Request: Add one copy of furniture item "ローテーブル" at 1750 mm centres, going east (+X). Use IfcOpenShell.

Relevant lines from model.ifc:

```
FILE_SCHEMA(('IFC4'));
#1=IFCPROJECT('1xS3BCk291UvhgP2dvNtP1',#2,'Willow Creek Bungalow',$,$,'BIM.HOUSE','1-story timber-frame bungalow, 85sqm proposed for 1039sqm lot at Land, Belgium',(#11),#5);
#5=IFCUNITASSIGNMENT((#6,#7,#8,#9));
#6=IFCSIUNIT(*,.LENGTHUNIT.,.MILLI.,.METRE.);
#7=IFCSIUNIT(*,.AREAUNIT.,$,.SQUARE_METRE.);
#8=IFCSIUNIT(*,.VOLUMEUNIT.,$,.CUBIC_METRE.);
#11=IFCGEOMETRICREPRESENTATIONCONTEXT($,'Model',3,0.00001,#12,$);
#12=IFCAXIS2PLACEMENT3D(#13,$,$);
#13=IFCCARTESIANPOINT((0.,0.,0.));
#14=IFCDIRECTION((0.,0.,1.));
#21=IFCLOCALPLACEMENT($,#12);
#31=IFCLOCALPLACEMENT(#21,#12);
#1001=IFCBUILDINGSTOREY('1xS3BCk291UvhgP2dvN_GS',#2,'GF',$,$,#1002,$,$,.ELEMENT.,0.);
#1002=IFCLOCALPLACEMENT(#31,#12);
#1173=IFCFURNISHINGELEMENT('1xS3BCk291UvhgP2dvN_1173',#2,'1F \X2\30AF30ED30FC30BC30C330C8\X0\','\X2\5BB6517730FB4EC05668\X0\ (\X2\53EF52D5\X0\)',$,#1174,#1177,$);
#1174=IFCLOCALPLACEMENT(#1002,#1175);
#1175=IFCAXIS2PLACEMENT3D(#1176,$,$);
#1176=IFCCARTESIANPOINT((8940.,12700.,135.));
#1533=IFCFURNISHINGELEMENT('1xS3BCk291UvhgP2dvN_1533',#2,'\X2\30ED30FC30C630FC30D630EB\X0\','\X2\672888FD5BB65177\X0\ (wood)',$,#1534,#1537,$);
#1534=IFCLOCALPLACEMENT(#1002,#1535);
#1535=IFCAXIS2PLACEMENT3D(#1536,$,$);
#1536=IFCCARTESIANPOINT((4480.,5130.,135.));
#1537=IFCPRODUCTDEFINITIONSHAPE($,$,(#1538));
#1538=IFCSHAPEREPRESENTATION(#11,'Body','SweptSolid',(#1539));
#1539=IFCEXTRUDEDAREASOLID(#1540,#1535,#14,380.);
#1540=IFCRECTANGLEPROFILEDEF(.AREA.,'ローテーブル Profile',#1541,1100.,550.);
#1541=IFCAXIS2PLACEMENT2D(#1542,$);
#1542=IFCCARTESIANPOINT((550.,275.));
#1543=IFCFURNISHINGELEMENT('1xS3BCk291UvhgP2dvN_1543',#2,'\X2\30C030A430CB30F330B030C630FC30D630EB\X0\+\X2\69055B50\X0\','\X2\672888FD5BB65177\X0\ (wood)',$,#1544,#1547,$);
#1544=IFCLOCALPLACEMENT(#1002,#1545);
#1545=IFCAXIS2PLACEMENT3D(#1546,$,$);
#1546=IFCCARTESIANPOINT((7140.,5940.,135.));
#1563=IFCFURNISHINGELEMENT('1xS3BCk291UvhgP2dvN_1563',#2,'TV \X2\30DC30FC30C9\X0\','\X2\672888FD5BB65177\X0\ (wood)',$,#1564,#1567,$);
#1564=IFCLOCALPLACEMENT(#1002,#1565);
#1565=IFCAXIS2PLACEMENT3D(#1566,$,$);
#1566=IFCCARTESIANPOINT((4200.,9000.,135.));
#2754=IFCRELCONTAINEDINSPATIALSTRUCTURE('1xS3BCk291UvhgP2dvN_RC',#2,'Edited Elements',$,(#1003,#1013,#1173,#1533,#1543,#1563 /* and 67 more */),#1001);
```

```python
import numpy as np
import ifcopenshell
import ifcopenshell.api.geometry
import ifcopenshell.api.root
import ifcopenshell.util.element
import ifcopenshell.util.placement

model = ifcopenshell.open("model.ifc")


def reuse_history(source, copy):
    """copy_class also copies each property set's owner history, people and application; keep the originals."""
    for rel in copy.IsDefinedBy:
        if rel.is_a("IfcRelDefinesByProperties") and (history := rel.RelatingPropertyDefinition.OwnerHistory):
            rel.RelatingPropertyDefinition.OwnerHistory = source.OwnerHistory
            ifcopenshell.util.element.remove_deep2(model, history)


source = model.by_id(1533)
base = ifcopenshell.util.placement.get_local_placement(source.ObjectPlacement)
step = np.array([1.0, 0.0, 0.0]) * 1750.0

for i in range(1, 2):
    copy = ifcopenshell.api.root.copy_class(model, product=source)
    copy.Representation = ifcopenshell.util.element.copy_deep(
        model, source.Representation, exclude=["IfcGeometricRepresentationContext", "IfcRepresentationMap"]
    )
    reuse_history(source, copy)
    matrix = base.copy()
    matrix[:3, 3] += i * step
    print("added at", matrix[:3, 3].round(3) + 0.0)
    ifcopenshell.api.geometry.edit_object_placement(model, product=copy, matrix=matrix, is_si=False)

model.write("model-out.ifc")
```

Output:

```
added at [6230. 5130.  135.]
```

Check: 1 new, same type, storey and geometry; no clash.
